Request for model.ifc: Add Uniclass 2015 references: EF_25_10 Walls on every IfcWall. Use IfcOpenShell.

First a look at what the model holds.

```python
import ifcopenshell

model = ifcopenshell.open("model.ifc")
print(model.schema)
print("classifications:", [c.Name for c in model.by_type("IfcClassification")])
for ifc_class in ("IfcDoor", "IfcRoof", "IfcStair", "IfcWall", "IfcWindow"):
    print(ifc_class, len(model.by_type(ifc_class)))
```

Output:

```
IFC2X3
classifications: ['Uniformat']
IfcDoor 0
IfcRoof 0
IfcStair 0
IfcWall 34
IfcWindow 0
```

```python
import ifcopenshell
import ifcopenshell.api.classification

model = ifcopenshell.open("model.ifc")

# IFC2X3 requires Source and Edition and has no link from the project to the system.
system = model.create_entity("IfcClassification", Source="NBS", Edition="2015", Name="Uniclass 2015")

codes = {
    "IfcWall": ("EF_25_10", "Walls"),
}
for ifc_class, (code, name) in codes.items():
    products = model.by_type(ifc_class)
    ifcopenshell.api.classification.add_reference(
        model, products=products, classification=system, identification=code, name=name
    )
    print(code, len(products))

model.write("model_edited.ifc")
```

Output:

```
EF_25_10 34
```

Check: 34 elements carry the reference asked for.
